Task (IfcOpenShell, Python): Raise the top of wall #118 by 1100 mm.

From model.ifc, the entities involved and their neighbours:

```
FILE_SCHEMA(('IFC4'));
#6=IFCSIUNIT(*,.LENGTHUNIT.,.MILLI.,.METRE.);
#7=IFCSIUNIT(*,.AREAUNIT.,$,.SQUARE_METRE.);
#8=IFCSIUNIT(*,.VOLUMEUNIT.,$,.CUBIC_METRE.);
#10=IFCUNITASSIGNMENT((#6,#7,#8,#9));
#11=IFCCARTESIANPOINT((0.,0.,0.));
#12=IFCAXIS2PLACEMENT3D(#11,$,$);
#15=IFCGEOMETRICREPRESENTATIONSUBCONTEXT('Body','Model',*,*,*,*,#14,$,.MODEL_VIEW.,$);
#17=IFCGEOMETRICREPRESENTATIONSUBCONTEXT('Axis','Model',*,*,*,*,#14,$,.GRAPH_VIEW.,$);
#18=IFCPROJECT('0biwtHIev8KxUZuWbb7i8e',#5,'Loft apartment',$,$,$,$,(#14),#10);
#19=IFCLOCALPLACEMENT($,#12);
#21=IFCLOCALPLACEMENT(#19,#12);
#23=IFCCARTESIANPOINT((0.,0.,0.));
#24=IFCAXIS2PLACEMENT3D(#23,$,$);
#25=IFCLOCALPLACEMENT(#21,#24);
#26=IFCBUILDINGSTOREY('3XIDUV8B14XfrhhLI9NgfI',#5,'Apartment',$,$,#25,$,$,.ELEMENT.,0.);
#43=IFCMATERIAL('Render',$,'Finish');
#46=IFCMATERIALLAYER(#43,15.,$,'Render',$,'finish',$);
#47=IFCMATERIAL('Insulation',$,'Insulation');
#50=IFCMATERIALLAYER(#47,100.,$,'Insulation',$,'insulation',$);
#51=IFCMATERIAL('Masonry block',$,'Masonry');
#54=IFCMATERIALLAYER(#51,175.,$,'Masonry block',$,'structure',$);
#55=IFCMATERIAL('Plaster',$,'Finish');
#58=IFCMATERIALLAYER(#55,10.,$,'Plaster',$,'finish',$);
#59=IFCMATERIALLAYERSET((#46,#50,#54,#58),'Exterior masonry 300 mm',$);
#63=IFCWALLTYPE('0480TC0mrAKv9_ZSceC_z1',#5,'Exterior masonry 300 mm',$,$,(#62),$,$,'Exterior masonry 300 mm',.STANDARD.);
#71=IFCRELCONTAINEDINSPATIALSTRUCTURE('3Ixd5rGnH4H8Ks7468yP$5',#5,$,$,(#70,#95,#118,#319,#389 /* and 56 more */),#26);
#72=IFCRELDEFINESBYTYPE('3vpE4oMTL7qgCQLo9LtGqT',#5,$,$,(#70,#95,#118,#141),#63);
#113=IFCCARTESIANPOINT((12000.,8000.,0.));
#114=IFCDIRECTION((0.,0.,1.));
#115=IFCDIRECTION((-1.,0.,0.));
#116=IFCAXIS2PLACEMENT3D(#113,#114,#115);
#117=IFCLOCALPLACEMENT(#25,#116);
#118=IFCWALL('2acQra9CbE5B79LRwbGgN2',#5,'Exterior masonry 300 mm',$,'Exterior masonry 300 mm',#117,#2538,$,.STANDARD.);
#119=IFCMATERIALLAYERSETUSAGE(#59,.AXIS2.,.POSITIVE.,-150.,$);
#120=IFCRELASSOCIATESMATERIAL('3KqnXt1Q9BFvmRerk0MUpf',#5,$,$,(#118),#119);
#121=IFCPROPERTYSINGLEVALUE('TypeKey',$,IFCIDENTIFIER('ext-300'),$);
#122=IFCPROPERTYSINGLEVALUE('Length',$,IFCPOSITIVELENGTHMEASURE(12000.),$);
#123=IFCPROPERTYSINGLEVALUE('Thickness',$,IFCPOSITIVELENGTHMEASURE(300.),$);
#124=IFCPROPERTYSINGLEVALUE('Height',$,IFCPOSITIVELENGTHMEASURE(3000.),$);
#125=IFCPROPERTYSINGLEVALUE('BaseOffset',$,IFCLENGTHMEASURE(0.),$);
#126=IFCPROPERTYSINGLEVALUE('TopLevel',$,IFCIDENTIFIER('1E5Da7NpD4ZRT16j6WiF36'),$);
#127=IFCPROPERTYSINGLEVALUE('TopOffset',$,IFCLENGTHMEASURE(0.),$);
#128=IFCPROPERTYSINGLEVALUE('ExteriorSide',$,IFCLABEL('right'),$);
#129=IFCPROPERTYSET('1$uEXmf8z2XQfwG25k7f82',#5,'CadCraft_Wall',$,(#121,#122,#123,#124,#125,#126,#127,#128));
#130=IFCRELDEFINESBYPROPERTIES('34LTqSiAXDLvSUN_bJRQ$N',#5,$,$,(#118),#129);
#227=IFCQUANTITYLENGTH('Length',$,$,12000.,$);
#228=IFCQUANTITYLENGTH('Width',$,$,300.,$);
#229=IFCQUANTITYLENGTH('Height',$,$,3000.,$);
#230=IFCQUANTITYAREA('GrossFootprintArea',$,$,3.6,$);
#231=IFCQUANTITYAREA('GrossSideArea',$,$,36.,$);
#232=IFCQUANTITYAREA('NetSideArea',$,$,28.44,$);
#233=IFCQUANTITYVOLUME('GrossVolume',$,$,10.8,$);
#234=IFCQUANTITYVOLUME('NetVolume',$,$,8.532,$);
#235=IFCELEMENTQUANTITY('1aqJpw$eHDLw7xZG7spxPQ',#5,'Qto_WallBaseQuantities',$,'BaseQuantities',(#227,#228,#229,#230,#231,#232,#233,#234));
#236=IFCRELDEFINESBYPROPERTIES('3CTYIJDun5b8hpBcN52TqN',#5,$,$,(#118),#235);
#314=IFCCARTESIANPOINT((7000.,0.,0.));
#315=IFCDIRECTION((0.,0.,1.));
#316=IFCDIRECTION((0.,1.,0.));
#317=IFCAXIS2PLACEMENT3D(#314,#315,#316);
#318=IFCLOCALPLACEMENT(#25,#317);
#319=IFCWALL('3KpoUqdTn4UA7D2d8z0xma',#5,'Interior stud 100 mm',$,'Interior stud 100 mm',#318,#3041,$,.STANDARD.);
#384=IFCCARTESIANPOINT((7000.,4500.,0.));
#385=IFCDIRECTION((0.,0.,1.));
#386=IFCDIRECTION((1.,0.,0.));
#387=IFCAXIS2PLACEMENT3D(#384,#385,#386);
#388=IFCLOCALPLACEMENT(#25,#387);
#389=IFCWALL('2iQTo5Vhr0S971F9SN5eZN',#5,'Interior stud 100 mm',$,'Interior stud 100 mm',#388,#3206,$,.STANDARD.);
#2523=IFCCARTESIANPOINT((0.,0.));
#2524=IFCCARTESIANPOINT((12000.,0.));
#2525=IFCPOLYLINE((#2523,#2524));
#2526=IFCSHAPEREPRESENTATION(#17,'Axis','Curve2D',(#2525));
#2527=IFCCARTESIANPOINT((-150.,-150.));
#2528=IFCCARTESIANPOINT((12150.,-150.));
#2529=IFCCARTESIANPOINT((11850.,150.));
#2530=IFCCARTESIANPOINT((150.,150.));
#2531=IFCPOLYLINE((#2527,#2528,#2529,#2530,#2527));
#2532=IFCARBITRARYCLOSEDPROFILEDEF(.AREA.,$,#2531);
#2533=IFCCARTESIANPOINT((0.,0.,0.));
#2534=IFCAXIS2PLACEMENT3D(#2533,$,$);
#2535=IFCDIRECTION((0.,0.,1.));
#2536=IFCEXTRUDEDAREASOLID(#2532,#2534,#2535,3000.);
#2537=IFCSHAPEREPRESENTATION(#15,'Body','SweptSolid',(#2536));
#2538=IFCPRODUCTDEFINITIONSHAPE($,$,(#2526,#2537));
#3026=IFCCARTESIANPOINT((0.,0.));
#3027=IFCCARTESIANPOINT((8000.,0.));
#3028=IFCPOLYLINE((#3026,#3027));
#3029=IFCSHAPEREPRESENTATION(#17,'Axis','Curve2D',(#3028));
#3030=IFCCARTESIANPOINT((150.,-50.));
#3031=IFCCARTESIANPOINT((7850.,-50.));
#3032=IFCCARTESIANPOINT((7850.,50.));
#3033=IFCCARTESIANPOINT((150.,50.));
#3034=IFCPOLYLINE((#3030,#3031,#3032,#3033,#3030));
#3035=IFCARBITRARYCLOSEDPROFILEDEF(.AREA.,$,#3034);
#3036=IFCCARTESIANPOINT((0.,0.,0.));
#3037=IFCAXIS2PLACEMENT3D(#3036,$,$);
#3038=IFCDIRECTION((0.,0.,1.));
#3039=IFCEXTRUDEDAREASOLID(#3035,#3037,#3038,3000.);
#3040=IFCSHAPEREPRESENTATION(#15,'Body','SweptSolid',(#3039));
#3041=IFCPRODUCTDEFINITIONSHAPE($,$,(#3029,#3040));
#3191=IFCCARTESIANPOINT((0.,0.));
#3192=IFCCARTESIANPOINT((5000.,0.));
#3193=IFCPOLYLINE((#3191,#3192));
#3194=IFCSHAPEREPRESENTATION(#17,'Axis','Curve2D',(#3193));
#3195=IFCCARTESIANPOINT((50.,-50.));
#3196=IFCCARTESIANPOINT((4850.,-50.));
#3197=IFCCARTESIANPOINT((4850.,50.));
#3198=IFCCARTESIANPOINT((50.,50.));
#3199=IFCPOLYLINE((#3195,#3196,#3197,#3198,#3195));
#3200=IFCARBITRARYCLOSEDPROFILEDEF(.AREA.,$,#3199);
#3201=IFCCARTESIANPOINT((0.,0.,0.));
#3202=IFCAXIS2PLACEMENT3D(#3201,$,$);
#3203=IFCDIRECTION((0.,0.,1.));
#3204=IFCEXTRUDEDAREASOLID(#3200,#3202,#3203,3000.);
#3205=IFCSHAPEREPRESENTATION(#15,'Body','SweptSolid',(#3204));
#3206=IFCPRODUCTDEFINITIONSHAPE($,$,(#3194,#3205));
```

```python
import ifcopenshell
import ifcopenshell.api.pset
import ifcopenshell.geom
import ifcopenshell.util.element
import ifcopenshell.util.representation
import ifcopenshell.util.shape
import ifcopenshell.util.unit

model = ifcopenshell.open("model.ifc")
unit_scale = ifcopenshell.util.unit.calculate_unit_scale(model)
area_scale = ifcopenshell.util.unit.calculate_unit_scale(model, "AREAUNIT")
volume_scale = ifcopenshell.util.unit.calculate_unit_scale(model, "VOLUMEUNIT")
settings = ifcopenshell.geom.settings()


def volume(element):
    """Net volume in cubic metres, openings subtracted."""
    shape = ifcopenshell.geom.create_shape(settings, element)
    return ifcopenshell.util.shape.get_volume(shape.geometry)


wall = model.by_guid("2acQra9CbE5B79LRwbGgN2")
before = volume(wall)

body = ifcopenshell.util.representation.get_representation(wall, "Model", "Body")
solid = body.Items[0]
old_height = solid.Depth
solid.Depth += 1.1 / unit_scale
after = volume(wall)
thickness = 0.3  # wall thickness in metres

# Update the stored height, areas and volumes.
pset = model.by_id(ifcopenshell.util.element.get_pset(wall, "CadCraft_Wall", should_inherit=False)["id"])
ifcopenshell.api.pset.edit_pset(model, pset=pset, properties={
    "Height": model.create_entity("IfcPositiveLengthMeasure", solid.Depth),
})
qto = model.by_id(ifcopenshell.util.element.get_pset(wall, "Qto_WallBaseQuantities", should_inherit=False)["id"])
ifcopenshell.api.pset.edit_qto(model, qto=qto, properties={
    "Height": solid.Depth,
    "GrossSideArea": ifcopenshell.util.element.get_pset(wall, "Qto_WallBaseQuantities", "GrossSideArea") * solid.Depth / old_height,
    "NetSideArea": after / thickness / area_scale,
    "GrossVolume": ifcopenshell.util.element.get_pset(wall, "Qto_WallBaseQuantities", "GrossVolume") * solid.Depth / old_height,
    "NetVolume": after / volume_scale,
})

print(f"height {old_height:g} -> {solid.Depth:g}, volume {before:.3f} -> {after:.3f} m3")

model.write("model_edited.ifc")
```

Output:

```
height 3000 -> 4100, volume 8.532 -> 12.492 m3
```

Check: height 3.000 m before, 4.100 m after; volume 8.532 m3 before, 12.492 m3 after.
